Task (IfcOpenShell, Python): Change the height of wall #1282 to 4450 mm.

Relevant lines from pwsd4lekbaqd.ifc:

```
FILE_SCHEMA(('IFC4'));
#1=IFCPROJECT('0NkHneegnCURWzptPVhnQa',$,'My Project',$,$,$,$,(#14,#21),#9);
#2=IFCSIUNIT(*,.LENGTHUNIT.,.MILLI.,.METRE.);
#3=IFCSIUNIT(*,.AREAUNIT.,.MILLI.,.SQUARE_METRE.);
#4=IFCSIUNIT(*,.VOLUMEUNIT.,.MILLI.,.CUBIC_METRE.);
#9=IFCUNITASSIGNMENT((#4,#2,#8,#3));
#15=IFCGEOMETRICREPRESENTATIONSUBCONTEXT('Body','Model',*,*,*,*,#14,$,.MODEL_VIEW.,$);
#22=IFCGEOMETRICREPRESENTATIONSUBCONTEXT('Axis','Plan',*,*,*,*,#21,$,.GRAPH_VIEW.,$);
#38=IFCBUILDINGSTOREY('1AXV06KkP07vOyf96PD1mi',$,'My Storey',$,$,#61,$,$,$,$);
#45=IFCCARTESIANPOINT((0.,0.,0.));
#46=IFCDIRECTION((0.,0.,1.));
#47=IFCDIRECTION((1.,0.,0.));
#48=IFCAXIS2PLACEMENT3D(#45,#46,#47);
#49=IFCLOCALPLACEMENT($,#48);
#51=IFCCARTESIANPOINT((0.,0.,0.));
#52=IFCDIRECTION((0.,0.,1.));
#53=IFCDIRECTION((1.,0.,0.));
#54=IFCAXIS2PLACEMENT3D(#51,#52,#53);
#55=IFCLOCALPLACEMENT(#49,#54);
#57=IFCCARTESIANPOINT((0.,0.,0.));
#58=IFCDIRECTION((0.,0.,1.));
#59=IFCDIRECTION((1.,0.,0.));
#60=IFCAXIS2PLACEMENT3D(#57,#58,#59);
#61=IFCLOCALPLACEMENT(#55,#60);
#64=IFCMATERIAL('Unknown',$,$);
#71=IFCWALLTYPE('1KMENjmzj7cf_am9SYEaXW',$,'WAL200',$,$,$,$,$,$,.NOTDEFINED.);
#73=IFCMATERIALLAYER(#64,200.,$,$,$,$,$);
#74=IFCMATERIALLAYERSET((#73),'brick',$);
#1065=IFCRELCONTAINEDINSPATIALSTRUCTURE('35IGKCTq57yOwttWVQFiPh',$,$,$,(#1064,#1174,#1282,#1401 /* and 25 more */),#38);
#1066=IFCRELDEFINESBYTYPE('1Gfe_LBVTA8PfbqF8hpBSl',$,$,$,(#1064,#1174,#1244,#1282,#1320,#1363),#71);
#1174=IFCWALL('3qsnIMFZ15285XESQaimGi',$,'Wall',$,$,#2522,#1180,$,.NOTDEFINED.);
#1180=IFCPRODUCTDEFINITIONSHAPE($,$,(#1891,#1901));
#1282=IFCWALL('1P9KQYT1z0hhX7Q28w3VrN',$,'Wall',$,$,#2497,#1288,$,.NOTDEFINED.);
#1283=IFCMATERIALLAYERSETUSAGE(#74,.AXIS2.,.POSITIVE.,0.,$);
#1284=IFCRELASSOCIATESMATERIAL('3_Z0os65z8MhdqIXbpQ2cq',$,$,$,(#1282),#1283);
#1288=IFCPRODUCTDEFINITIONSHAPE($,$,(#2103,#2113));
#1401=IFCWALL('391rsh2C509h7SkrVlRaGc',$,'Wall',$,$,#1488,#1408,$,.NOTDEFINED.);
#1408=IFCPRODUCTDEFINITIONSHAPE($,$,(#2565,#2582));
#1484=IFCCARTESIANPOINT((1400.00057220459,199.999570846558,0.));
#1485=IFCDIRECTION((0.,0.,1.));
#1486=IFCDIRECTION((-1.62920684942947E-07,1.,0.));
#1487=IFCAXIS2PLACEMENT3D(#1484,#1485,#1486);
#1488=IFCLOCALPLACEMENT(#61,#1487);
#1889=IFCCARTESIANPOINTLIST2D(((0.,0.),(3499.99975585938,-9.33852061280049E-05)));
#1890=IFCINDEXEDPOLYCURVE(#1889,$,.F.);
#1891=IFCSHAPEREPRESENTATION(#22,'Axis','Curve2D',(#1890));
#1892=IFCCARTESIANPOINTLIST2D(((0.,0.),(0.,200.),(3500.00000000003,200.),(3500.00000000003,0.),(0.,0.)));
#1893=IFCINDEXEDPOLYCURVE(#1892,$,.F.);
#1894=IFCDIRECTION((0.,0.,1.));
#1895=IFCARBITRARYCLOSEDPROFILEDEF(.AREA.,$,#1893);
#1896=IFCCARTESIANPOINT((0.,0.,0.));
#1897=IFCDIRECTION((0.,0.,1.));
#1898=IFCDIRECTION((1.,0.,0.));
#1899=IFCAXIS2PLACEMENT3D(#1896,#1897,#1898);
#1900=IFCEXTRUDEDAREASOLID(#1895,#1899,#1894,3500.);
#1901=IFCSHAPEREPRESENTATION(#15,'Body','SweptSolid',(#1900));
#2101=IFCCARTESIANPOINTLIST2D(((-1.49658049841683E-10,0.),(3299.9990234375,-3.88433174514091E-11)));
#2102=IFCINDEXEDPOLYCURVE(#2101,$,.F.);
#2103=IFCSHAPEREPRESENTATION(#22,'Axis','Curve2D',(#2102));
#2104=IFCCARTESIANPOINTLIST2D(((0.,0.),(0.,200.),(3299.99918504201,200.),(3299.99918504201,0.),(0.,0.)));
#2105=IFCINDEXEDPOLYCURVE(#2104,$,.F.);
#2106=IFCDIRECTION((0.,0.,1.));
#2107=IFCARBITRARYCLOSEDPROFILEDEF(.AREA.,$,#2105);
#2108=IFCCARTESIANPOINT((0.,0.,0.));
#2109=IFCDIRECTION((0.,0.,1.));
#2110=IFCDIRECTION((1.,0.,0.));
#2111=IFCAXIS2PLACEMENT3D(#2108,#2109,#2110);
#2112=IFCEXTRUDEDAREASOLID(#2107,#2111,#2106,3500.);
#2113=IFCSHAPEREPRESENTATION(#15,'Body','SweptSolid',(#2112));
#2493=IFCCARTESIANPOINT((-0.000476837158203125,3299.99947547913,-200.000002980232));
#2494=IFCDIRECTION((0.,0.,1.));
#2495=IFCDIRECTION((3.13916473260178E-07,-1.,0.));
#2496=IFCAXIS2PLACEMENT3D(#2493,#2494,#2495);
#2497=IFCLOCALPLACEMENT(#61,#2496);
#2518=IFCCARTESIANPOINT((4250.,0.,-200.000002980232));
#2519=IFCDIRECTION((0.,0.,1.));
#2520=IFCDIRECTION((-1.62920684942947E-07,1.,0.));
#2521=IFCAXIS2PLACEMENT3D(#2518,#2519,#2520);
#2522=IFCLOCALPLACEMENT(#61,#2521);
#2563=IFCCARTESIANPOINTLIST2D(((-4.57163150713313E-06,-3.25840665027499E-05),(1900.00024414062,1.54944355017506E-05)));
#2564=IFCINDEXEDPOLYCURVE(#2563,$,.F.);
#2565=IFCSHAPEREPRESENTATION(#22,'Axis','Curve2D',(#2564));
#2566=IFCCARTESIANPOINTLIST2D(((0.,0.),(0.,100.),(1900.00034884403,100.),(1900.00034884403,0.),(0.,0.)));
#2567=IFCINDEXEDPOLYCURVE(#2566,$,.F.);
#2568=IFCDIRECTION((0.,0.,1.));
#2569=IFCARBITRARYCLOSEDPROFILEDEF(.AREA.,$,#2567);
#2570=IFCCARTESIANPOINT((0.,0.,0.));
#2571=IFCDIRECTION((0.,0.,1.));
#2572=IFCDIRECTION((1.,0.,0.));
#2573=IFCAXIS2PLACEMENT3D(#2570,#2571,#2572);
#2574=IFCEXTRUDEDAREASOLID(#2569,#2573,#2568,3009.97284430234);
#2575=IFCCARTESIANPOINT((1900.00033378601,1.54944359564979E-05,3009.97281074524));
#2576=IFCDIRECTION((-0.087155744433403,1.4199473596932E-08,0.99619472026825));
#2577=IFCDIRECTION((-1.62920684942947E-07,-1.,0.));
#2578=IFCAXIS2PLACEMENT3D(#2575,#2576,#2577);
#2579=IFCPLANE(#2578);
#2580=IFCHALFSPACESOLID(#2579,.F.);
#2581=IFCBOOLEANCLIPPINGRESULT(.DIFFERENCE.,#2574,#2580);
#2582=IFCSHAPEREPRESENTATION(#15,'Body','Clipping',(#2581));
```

```python
import ifcopenshell
import ifcopenshell.geom
import ifcopenshell.util.representation
import ifcopenshell.util.shape
import ifcopenshell.util.unit

model = ifcopenshell.open("pwsd4lekbaqd.ifc")
unit_scale = ifcopenshell.util.unit.calculate_unit_scale(model)
settings = ifcopenshell.geom.settings()


def volume(element):
    """Net volume in cubic metres, openings subtracted."""
    shape = ifcopenshell.geom.create_shape(settings, element)
    return ifcopenshell.util.shape.get_volume(shape.geometry)


wall = model.by_guid("1P9KQYT1z0hhX7Q28w3VrN")
before = volume(wall)

body = ifcopenshell.util.representation.get_representation(wall, "Model", "Body")
solid = body.Items[0]
old_height = solid.Depth
solid.Depth = 4.45 / unit_scale
after = volume(wall)

print(f"height {old_height:g} -> {solid.Depth:g}, volume {before:.3f} -> {after:.3f} m3")

model.write("pwsd4lekbaqd_updated.ifc")
```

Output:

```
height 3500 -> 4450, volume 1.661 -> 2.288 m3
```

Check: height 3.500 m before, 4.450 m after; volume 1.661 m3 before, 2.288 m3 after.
